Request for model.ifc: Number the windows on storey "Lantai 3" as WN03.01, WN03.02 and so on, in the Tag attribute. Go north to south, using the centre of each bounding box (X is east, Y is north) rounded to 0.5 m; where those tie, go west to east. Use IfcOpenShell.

First a look at what the model holds.

```python
import ifcopenshell
import ifcopenshell.util.element
import ifcopenshell.util.placement

model = ifcopenshell.open("model.ifc")
print(model.schema)
storey = next(s for s in model.by_type("IfcBuildingStorey") if s.Name == "Lantai 3")
windows = [e for e in ifcopenshell.util.element.get_decomposition(storey) if e.is_a("IfcWindow")]
for e in sorted(windows, key=lambda e: e.id()):
    origin = ifcopenshell.util.placement.get_local_placement(e.ObjectPlacement)[:3, 3]
    print(e.id(), e.Tag, e.Name, origin.round(2) + 0.0, sep=" | ")
```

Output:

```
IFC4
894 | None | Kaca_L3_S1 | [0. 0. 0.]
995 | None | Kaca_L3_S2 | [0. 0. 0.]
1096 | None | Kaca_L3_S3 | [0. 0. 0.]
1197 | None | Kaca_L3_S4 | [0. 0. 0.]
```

```python
import ifcopenshell
import ifcopenshell.geom
import ifcopenshell.util.element
import ifcopenshell.util.shape

model = ifcopenshell.open("model.ifc")
settings = ifcopenshell.geom.settings()
settings.set("use-world-coords", True)


def centre(element):
    shape = ifcopenshell.geom.create_shape(settings, element)
    return ifcopenshell.util.shape.get_bbox_centroid(shape.geometry)


storey = next(s for s in model.by_type("IfcBuildingStorey") if s.Name == "Lantai 3")
windows = [e for e in ifcopenshell.util.element.get_decomposition(storey) if e.is_a("IfcWindow")]

# Insertion points can sit at a corner or the storey origin, so sort by the geometry (in metres).
centres = {e: centre(e) for e in windows}
windows.sort(key=lambda e: (-round(centres[e][1] / 0.5), centres[e][0]))

for i, e in enumerate(windows, start=1):
    number = f"WN03.{i:02d}"
    e.Tag = number
    print(e.id(), number)

model.write("model-out.ifc")
```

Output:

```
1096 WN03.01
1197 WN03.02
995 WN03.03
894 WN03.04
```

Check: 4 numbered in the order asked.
